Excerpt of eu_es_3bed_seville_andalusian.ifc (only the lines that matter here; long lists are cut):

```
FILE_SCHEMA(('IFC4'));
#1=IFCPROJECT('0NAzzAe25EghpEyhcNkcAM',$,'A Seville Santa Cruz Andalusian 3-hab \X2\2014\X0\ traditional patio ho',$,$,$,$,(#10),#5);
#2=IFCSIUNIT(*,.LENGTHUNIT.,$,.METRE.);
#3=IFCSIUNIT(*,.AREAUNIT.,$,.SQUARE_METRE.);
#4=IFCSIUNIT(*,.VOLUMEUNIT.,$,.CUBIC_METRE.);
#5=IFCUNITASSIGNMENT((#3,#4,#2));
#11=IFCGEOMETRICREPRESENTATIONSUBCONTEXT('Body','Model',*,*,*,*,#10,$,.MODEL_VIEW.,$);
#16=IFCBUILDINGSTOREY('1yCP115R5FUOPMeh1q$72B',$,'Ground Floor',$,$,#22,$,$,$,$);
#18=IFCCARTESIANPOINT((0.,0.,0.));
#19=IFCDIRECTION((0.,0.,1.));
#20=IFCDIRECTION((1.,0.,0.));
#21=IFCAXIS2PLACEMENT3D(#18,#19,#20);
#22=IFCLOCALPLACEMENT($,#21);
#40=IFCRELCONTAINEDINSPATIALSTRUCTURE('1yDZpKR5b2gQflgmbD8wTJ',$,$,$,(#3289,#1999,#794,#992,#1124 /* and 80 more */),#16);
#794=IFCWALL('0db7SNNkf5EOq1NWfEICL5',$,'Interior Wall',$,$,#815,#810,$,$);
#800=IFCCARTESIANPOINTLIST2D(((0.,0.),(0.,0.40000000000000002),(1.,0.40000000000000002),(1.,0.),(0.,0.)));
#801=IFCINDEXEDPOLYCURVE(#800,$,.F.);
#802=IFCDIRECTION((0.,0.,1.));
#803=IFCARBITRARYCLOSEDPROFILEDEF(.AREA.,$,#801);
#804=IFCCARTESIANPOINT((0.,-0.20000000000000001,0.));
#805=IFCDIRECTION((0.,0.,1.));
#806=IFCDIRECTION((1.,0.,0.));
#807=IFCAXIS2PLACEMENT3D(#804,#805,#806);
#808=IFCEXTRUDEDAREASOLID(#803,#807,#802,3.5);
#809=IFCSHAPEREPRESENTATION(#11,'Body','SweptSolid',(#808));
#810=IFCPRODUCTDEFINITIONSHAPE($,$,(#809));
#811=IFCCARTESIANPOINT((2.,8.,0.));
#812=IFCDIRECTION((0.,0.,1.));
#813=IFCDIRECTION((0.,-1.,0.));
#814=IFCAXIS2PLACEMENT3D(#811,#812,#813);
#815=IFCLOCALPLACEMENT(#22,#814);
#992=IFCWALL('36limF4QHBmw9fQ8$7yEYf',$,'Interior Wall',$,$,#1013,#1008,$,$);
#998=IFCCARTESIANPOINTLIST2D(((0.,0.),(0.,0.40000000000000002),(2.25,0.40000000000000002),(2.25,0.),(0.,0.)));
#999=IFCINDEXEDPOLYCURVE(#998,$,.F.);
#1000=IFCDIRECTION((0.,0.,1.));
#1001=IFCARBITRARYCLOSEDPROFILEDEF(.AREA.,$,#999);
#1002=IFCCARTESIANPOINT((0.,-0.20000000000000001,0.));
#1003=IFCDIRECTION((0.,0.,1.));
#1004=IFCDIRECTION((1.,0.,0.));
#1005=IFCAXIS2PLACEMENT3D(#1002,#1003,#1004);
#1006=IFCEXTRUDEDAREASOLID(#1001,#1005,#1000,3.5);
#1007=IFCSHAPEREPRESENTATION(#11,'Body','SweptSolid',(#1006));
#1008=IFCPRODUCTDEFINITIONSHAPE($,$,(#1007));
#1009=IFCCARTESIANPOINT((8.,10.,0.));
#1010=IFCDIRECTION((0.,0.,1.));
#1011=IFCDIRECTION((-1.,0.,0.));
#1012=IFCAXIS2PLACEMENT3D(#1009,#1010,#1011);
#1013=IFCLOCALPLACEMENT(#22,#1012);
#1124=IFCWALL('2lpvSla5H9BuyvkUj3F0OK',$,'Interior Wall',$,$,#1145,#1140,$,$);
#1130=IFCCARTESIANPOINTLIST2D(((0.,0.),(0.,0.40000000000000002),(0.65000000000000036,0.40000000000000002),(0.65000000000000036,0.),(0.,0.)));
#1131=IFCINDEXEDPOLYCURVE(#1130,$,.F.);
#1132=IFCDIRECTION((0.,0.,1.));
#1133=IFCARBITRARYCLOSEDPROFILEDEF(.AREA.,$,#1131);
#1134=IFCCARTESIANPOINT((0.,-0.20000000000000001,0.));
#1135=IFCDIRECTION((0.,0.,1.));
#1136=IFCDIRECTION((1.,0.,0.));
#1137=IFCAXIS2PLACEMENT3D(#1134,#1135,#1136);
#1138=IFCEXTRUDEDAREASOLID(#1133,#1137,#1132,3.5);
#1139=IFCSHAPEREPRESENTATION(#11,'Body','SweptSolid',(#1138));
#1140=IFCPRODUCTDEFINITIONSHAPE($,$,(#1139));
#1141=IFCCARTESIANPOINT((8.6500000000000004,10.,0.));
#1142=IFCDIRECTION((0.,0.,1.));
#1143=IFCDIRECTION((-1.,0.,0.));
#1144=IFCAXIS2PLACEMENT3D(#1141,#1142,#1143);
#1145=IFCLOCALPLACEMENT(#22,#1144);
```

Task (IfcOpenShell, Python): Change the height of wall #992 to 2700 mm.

```python
import ifcopenshell
import ifcopenshell.geom
import ifcopenshell.util.representation
import ifcopenshell.util.shape
import ifcopenshell.util.unit

model = ifcopenshell.open("eu_es_3bed_seville_andalusian.ifc")
unit_scale = ifcopenshell.util.unit.calculate_unit_scale(model)
settings = ifcopenshell.geom.settings()


def volume(element):
    """Net volume in cubic metres, openings subtracted."""
    shape = ifcopenshell.geom.create_shape(settings, element)
    return ifcopenshell.util.shape.get_volume(shape.geometry)


wall = model.by_guid("36limF4QHBmw9fQ8$7yEYf")
before = volume(wall)

body = ifcopenshell.util.representation.get_representation(wall, "Model", "Body")
solid = body.Items[0]
old_height = solid.Depth
solid.Depth = 2.7 / unit_scale
after = volume(wall)

print(f"height {old_height:g} -> {solid.Depth:g}, volume {before:.3f} -> {after:.3f} m3")

model.write("eu_es_3bed_seville_andalusian_rev.ifc")
```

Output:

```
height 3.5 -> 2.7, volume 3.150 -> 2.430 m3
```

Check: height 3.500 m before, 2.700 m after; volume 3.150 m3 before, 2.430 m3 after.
